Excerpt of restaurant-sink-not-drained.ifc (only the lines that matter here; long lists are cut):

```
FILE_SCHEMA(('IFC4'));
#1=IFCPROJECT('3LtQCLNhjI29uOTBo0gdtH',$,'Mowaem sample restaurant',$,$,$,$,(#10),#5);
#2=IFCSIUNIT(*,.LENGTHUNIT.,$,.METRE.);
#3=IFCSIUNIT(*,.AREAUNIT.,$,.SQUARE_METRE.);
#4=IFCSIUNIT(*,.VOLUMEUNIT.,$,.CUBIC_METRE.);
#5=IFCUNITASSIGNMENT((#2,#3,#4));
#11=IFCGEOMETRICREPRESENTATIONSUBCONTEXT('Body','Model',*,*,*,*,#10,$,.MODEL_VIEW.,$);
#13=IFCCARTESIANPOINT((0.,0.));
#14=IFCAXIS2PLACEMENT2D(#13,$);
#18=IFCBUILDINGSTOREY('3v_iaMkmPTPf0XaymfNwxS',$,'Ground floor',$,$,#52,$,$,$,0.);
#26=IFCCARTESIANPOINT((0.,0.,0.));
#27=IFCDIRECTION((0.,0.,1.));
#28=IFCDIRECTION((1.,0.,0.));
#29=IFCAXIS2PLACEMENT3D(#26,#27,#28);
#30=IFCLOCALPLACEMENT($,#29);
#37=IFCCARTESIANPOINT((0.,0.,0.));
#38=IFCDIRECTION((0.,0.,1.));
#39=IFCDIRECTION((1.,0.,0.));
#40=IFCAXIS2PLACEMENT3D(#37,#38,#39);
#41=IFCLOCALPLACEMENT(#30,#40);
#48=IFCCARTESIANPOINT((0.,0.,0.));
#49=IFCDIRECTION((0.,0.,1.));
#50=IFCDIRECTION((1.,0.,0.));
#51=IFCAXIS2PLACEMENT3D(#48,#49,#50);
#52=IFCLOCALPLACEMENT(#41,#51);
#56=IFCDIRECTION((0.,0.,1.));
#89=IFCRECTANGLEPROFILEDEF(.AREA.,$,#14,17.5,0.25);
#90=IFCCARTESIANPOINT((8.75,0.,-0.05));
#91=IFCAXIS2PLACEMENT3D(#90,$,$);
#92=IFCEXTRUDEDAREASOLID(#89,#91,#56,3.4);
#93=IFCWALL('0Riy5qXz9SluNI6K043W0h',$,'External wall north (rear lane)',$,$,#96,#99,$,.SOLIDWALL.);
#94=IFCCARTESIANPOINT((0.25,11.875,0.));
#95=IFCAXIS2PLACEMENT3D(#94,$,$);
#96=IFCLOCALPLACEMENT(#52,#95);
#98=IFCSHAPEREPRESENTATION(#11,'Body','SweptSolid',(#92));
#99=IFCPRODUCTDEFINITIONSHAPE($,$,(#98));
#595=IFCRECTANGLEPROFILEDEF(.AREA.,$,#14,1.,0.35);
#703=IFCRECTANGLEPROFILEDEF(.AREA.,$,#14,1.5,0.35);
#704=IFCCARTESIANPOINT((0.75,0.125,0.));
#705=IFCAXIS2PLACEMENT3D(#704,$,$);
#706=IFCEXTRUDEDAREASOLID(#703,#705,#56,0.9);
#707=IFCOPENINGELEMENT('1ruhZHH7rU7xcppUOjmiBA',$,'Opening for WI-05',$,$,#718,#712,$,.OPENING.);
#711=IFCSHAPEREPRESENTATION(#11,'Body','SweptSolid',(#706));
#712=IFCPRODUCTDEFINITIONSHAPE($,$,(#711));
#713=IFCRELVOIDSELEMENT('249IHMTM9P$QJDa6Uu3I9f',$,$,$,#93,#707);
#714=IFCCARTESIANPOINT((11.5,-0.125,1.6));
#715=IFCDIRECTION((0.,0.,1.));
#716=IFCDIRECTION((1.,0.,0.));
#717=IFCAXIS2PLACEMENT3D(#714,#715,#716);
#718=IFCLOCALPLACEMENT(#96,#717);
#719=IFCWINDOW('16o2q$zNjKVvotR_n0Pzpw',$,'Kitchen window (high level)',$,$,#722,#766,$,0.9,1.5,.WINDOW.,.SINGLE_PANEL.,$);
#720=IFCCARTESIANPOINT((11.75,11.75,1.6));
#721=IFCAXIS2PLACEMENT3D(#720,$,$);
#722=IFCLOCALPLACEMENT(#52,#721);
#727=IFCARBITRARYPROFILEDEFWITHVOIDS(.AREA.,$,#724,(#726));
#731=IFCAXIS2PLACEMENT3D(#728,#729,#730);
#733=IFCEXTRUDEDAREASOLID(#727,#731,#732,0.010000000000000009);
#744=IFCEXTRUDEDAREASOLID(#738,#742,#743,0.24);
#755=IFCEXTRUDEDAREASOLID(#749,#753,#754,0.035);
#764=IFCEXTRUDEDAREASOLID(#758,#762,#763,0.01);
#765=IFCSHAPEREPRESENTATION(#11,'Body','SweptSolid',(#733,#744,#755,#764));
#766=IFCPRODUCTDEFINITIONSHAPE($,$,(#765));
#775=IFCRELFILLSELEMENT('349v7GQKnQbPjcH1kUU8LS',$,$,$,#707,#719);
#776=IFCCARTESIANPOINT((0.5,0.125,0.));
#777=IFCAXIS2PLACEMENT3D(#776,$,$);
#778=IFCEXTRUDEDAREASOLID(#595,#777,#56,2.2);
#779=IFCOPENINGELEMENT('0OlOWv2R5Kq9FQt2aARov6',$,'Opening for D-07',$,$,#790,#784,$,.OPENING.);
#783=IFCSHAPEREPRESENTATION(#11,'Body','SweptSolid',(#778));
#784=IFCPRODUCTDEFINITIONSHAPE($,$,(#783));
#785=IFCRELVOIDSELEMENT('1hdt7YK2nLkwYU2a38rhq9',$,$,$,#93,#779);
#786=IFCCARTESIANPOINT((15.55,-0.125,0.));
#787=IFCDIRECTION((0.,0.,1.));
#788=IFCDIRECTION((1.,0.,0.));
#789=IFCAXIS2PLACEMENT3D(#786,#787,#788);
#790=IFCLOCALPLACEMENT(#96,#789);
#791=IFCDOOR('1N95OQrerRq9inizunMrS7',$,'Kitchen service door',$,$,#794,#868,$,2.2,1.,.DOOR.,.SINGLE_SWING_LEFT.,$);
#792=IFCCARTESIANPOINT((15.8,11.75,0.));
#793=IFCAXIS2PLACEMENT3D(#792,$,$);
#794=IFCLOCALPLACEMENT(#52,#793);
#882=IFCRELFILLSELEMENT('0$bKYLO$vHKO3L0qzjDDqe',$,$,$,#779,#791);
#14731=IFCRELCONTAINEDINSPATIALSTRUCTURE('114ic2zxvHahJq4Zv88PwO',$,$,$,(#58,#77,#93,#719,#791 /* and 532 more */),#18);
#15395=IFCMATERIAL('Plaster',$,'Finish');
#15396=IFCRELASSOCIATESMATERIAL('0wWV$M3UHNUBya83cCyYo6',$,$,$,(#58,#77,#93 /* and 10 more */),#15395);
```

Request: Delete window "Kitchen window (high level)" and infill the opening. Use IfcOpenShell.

```python
import ifcopenshell
import ifcopenshell.api.feature
import ifcopenshell.api.root
import ifcopenshell.geom
import ifcopenshell.util.shape

model = ifcopenshell.open("restaurant-sink-not-drained.ifc")
settings = ifcopenshell.geom.settings()


def volume(element):
    """Net volume in cubic metres, openings subtracted."""
    shape = ifcopenshell.geom.create_shape(settings, element)
    return ifcopenshell.util.shape.get_volume(shape.geometry)


window = model.by_id(719)
opening = window.FillsVoids[0].RelatingOpeningElement
wall = opening.VoidsElements[0].RelatingBuildingElement
before = volume(wall)

ifcopenshell.api.root.remove_product(model, product=window)
ifcopenshell.api.feature.remove_feature(model, feature=opening)

after = volume(wall)

print(f"wall volume {before:.3f} -> {after:.3f} m3")

model.write("restaurant-sink-not-drained_updated.ifc")
```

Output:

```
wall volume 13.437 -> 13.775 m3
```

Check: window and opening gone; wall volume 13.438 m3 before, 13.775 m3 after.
